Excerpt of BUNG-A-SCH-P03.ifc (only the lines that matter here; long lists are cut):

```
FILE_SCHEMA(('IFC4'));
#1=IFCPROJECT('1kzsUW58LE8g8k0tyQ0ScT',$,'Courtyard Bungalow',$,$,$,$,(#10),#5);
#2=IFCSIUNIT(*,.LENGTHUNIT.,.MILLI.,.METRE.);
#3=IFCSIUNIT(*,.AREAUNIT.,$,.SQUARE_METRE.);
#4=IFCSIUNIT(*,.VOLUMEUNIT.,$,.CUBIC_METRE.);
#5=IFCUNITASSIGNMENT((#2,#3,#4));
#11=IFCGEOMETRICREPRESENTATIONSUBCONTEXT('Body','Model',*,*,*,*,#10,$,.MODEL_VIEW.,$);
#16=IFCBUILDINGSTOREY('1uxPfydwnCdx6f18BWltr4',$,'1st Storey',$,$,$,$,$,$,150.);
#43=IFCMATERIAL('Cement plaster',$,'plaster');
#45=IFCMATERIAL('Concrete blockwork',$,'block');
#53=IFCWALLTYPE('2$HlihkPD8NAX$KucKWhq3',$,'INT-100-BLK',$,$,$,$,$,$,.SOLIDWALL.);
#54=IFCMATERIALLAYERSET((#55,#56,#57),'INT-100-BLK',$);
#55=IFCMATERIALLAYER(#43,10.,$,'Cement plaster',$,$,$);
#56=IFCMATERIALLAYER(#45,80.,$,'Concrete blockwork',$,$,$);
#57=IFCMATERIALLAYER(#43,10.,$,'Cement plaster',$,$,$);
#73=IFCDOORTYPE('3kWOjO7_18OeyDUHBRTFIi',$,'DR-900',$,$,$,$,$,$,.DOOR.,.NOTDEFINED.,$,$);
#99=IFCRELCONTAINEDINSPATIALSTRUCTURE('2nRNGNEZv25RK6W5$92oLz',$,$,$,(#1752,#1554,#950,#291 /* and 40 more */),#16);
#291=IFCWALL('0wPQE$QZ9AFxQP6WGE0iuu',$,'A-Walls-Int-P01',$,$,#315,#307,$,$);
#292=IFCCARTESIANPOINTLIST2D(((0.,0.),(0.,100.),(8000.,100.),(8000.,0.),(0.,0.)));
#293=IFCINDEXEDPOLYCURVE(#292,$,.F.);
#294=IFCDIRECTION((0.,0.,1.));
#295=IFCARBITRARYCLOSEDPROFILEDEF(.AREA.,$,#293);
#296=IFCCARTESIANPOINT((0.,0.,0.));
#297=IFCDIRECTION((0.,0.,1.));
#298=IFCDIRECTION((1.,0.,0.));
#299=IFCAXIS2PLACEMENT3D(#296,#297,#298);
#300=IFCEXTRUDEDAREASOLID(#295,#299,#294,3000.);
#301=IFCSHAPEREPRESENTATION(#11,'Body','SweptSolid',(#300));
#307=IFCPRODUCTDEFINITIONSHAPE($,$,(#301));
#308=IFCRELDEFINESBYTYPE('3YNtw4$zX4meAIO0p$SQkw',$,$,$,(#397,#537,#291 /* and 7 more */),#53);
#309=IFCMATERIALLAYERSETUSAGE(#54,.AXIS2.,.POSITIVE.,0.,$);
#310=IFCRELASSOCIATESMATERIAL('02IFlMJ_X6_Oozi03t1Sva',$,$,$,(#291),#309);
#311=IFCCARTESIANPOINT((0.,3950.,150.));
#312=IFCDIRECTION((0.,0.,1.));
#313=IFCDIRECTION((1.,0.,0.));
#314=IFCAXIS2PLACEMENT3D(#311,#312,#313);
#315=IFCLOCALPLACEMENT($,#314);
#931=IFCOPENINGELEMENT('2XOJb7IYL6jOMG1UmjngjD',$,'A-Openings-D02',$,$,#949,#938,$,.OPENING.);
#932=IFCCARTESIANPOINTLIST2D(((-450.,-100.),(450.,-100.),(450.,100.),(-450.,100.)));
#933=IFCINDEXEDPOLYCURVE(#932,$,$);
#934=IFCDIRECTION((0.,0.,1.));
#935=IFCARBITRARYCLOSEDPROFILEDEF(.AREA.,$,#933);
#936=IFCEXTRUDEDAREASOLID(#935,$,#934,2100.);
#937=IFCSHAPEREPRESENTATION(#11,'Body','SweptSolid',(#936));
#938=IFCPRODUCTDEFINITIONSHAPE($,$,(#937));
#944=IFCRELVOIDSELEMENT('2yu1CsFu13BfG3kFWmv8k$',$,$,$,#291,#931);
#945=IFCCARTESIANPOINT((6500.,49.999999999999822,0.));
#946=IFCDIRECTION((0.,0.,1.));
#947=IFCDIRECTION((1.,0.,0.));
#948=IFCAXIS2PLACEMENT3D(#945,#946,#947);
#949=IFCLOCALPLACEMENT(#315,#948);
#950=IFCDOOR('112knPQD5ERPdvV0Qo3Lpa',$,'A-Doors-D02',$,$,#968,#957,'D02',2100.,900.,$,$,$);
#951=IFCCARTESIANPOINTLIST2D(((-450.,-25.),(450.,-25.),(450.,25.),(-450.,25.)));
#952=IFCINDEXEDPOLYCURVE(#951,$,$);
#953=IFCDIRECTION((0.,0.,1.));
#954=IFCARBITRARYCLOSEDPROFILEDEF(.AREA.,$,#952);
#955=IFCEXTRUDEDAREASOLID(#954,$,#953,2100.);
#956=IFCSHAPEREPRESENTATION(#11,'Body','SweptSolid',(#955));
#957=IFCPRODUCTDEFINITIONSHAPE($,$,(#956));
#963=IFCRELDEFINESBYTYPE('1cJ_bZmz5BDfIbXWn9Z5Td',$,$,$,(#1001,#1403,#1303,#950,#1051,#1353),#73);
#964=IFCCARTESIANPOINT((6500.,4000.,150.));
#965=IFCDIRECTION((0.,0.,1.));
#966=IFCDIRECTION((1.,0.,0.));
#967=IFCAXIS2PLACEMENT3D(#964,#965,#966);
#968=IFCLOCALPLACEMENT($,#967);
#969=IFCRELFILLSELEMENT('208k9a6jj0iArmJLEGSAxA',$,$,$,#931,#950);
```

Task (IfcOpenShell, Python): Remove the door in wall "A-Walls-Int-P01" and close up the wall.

```python
import ifcopenshell
import ifcopenshell.api.feature
import ifcopenshell.api.root
import ifcopenshell.geom
import ifcopenshell.util.shape

model = ifcopenshell.open("BUNG-A-SCH-P03.ifc")
settings = ifcopenshell.geom.settings()


def volume(element):
    """Net volume in cubic metres, openings subtracted."""
    shape = ifcopenshell.geom.create_shape(settings, element)
    return ifcopenshell.util.shape.get_volume(shape.geometry)


door = model.by_guid("112knPQD5ERPdvV0Qo3Lpa")
opening = door.FillsVoids[0].RelatingOpeningElement
wall = opening.VoidsElements[0].RelatingBuildingElement
before = volume(wall)

ifcopenshell.api.root.remove_product(model, product=door)
ifcopenshell.api.feature.remove_feature(model, feature=opening)

after = volume(wall)

print(f"wall volume {before:.3f} -> {after:.3f} m3")

model.write("BUNG-A-SCH-P03_v2.ifc")
```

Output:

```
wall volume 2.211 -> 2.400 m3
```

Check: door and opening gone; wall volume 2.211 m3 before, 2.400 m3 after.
